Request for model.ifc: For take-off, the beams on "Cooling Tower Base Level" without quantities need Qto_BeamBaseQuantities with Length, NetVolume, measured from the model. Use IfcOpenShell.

First a look at what the model holds.

```python
import ifcopenshell
import ifcopenshell.util.element
import ifcopenshell.util.unit

model = ifcopenshell.open("model.ifc")
print(model.schema)
for unit_type in ("LENGTHUNIT", "AREAUNIT", "VOLUMEUNIT"):
    print(unit_type, ifcopenshell.util.unit.calculate_unit_scale(model, unit_type))
storey = next(s for s in model.by_type("IfcBuildingStorey") if s.Name == "Cooling Tower Base Level")
beams = [e for e in ifcopenshell.util.element.get_decomposition(storey) if e.is_a("IfcBeam")]
for e in sorted(beams, key=lambda e: e.id()):
    print(e.id(), e.is_a(), e.Name, list(ifcopenshell.util.element.get_psets(e, qtos_only=True)), sep=" | ")
```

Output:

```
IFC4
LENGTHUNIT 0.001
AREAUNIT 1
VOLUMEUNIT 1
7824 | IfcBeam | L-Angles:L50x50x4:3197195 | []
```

```python
import ifcopenshell
import ifcopenshell.api.pset
import ifcopenshell.geom
import ifcopenshell.util.element
import ifcopenshell.util.shape
import ifcopenshell.util.unit

model = ifcopenshell.open("model.ifc")
unit_scale = ifcopenshell.util.unit.calculate_unit_scale(model)
volume_scale = ifcopenshell.util.unit.calculate_unit_scale(model, "VOLUMEUNIT")
settings = ifcopenshell.geom.settings()

storey = next(s for s in model.by_type("IfcBuildingStorey") if s.Name == "Cooling Tower Base Level")
beams = [e for e in ifcopenshell.util.element.get_decomposition(storey) if e.is_a("IfcBeam")]

for e in sorted(beams, key=lambda e: e.id()):
    if ifcopenshell.util.element.get_psets(e, qtos_only=True, should_inherit=False):
        continue
    # Geometry comes back in metres, in the element's own axes.
    shape = ifcopenshell.geom.create_shape(settings, e)
    values = {
        "Length": ifcopenshell.util.shape.get_max_xyz(shape.geometry) / unit_scale,
        "NetVolume": ifcopenshell.util.shape.get_volume(shape.geometry) / volume_scale,
    }
    qto = ifcopenshell.api.pset.add_qto(model, product=e, name="Qto_BeamBaseQuantities")
    ifcopenshell.api.pset.edit_qto(model, qto=qto, properties=values)
    print(e.id(), {k: round(v, 3) for k, v in values.items()})

model.write("model_edited.ifc")
```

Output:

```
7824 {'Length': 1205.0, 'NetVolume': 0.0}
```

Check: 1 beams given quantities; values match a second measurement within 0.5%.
